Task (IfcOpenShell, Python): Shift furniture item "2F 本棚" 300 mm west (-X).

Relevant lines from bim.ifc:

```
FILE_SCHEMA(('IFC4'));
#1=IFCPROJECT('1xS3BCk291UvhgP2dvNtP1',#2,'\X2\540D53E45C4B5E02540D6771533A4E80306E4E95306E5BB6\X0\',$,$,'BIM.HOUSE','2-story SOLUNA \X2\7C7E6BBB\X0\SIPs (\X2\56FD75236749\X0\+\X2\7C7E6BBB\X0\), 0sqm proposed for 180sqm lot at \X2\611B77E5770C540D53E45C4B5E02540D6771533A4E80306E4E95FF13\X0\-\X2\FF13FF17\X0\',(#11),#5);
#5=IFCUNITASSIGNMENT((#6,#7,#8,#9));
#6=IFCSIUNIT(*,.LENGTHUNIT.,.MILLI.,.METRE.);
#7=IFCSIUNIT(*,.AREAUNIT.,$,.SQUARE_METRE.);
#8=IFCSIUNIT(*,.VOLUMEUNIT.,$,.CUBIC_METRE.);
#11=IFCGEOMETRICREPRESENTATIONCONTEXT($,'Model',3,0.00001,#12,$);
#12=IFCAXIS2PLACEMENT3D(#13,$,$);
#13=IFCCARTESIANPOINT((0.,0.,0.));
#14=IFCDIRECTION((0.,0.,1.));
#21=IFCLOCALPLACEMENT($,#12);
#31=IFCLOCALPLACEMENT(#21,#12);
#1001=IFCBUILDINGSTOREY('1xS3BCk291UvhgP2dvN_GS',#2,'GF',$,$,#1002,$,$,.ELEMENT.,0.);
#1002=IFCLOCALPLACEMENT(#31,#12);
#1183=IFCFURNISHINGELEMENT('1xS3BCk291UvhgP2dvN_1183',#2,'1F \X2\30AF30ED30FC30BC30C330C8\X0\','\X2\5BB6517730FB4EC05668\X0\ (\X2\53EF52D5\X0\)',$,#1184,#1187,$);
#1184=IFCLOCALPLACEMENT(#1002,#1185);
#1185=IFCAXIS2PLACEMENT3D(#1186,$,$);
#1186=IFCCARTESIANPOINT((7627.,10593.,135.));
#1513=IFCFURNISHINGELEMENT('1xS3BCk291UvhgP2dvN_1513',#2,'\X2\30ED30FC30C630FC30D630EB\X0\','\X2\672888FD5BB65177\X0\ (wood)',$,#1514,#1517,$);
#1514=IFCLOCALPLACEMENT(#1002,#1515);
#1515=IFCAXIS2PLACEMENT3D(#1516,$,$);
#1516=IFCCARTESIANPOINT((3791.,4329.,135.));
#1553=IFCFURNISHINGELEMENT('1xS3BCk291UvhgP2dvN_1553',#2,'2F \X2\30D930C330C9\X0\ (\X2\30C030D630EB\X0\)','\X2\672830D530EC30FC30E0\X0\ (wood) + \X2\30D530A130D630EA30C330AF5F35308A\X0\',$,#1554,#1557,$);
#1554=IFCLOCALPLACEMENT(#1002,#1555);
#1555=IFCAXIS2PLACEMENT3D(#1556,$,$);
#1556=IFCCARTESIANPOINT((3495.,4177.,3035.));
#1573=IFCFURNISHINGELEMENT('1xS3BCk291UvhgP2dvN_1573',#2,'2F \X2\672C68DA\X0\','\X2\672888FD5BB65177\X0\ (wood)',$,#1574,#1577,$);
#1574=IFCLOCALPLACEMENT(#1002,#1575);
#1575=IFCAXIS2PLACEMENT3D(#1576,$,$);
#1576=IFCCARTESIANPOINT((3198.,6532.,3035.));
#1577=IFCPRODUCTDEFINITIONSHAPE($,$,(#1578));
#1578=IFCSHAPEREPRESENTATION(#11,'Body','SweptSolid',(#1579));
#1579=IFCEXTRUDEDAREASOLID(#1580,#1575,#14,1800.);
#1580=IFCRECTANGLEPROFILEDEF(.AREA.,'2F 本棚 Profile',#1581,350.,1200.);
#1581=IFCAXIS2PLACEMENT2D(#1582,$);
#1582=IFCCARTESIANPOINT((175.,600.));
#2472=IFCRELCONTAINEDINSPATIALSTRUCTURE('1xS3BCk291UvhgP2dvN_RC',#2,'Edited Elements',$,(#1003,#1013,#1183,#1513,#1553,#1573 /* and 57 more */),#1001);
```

```python
import ifcopenshell
import ifcopenshell.api.geometry
import ifcopenshell.util.placement
import ifcopenshell.util.unit

model = ifcopenshell.open("bim.ifc")
unit_scale = ifcopenshell.util.unit.calculate_unit_scale(model)

item = model.by_guid("1xS3BCk291UvhgP2dvN_1573")
matrix = ifcopenshell.util.placement.get_local_placement(item.ObjectPlacement)
matrix[0, 3] -= 0.3 / unit_scale
ifcopenshell.api.geometry.edit_object_placement(model, product=item, matrix=matrix, is_si=False)

print(ifcopenshell.util.placement.get_local_placement(item.ObjectPlacement).round(3) + 0.0)

model.write("bim_rev.ifc")
```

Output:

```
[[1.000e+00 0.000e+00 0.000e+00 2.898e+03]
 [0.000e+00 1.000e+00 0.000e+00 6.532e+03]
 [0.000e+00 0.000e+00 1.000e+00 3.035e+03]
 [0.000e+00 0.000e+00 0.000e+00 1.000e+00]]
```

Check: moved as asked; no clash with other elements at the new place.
